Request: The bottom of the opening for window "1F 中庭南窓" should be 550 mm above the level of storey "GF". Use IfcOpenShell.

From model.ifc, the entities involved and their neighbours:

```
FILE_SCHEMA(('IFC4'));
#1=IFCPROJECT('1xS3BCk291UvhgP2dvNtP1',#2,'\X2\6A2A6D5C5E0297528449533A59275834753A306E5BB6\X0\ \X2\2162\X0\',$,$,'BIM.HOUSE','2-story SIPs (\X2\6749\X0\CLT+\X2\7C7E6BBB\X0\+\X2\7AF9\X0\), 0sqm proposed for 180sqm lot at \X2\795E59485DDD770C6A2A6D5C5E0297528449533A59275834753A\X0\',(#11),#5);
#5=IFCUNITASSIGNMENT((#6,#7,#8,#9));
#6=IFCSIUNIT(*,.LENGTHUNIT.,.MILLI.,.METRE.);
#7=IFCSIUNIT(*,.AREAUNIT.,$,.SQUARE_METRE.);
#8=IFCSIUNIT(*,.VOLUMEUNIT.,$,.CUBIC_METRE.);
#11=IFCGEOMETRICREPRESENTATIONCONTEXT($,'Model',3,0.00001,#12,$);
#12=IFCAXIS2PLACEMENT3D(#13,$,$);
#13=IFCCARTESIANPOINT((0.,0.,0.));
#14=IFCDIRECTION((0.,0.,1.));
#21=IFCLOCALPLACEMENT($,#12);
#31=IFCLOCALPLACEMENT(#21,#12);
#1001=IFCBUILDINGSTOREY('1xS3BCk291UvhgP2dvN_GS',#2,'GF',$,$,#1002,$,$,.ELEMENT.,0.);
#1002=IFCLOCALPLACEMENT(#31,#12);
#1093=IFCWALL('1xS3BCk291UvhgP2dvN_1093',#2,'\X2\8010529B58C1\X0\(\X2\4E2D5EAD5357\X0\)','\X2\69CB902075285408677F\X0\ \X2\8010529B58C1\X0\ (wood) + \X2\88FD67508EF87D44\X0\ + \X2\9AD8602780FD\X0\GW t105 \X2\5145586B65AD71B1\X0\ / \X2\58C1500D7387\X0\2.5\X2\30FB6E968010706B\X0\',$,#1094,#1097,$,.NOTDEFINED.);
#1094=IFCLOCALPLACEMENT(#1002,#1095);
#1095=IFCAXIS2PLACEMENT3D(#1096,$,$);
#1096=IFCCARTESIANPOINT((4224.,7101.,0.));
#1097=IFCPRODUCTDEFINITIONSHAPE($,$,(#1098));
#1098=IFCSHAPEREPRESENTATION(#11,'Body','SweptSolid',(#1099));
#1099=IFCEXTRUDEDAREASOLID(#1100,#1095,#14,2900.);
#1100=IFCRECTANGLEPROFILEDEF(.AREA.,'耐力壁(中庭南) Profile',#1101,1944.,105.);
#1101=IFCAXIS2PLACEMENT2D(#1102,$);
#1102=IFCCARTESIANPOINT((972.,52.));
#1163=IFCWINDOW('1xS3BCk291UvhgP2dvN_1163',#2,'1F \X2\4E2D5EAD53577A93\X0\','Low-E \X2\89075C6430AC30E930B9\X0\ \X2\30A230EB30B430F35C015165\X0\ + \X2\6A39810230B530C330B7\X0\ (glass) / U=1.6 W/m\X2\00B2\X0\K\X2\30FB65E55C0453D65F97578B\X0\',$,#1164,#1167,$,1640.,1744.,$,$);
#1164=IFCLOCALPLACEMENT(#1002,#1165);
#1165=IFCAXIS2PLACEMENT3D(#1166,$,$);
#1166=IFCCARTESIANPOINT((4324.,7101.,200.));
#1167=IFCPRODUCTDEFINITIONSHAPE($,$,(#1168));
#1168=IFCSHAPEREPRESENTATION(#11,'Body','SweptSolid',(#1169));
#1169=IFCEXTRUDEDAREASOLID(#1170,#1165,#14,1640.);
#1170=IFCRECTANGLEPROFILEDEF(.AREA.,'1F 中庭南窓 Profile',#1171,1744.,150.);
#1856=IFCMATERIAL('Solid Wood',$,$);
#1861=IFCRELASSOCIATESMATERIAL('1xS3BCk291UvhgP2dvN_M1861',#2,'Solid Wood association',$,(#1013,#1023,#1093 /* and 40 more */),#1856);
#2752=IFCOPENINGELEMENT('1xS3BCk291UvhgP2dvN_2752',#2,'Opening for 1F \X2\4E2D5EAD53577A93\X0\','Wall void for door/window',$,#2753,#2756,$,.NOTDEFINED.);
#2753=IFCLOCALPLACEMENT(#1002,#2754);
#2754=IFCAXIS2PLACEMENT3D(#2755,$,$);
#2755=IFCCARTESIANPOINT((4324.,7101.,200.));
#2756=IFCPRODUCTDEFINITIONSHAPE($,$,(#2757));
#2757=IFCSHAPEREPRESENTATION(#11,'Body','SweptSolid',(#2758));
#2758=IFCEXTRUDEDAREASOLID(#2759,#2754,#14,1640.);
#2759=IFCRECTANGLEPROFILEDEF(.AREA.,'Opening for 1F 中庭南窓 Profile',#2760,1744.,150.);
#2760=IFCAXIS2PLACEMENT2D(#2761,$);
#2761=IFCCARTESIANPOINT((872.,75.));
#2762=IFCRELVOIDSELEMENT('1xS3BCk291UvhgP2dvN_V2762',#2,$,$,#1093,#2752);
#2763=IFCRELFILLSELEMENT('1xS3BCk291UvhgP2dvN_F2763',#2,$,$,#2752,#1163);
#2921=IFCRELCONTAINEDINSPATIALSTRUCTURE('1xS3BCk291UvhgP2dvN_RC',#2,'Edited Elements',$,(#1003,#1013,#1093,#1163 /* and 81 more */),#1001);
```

```python
import numpy as np
import ifcopenshell
import ifcopenshell.api.geometry
import ifcopenshell.geom
import ifcopenshell.util.element
import ifcopenshell.util.placement
import ifcopenshell.util.shape
import ifcopenshell.util.unit

model = ifcopenshell.open("model.ifc")
unit_scale = ifcopenshell.util.unit.calculate_unit_scale(model)

window = model.by_id(1163)
opening = window.FillsVoids[0].RelatingOpeningElement
storey = ifcopenshell.util.element.get_container(window, ifc_class="IfcBuildingStorey")
level = ifcopenshell.util.placement.get_local_placement(storey.ObjectPlacement)[2, 3]

# The opening's origin need not be at the sill, so measure its lowest point.
shape = ifcopenshell.geom.create_shape(ifcopenshell.geom.settings(), opening)
bottom = ifcopenshell.util.shape.get_shape_bottom_elevation(shape, shape.geometry) / unit_scale
dz = level + 550.0 - bottom

shift = np.array([0.0, 0.0, dz])
# The window is not placed relative to its opening, so move both.
for product in (opening, window):
    matrix = ifcopenshell.util.placement.get_local_placement(product.ObjectPlacement)
    matrix[:3, 3] += shift
    ifcopenshell.api.geometry.edit_object_placement(model, product=product, matrix=matrix, is_si=False)

print(f"moved by {dz * unit_scale:+.3f} m")

model.write("model_rev.ifc")
```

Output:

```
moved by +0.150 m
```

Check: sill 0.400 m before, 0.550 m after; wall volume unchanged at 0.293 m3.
